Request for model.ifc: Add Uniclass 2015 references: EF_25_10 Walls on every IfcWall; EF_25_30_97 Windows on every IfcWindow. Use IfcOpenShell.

First a look at what the model holds.

```python
import ifcopenshell

model = ifcopenshell.open("model.ifc")
print(model.schema)
print("classifications:", [c.Name for c in model.by_type("IfcClassification")])
for ifc_class in ("IfcDoor", "IfcRoof", "IfcStair", "IfcWall", "IfcWindow"):
    print(ifc_class, len(model.by_type(ifc_class)))
```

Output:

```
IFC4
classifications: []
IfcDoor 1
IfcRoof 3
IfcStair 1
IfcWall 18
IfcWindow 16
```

```python
import ifcopenshell
import ifcopenshell.api.classification

model = ifcopenshell.open("model.ifc")

system = ifcopenshell.api.classification.add_classification(model, classification="Uniclass 2015")

codes = {
    "IfcWall": ("EF_25_10", "Walls"),
    "IfcWindow": ("EF_25_30_97", "Windows"),
}
for ifc_class, (code, name) in codes.items():
    products = model.by_type(ifc_class)
    ifcopenshell.api.classification.add_reference(
        model, products=products, classification=system, identification=code, name=name
    )
    print(code, len(products))

model.write("model_updated.ifc")
```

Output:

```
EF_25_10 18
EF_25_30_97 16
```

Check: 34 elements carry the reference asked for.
